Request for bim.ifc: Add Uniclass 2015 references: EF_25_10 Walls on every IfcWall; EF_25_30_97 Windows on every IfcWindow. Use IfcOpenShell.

First a look at what the model holds.

```python
import ifcopenshell

model = ifcopenshell.open("bim.ifc")
print(model.schema)
print("classifications:", [c.Name for c in model.by_type("IfcClassification")])
for ifc_class in ("IfcDoor", "IfcRoof", "IfcStair", "IfcWall", "IfcWindow"):
    print(ifc_class, len(model.by_type(ifc_class)))
```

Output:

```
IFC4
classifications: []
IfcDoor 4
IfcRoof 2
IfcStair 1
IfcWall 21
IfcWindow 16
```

```python
import ifcopenshell
import ifcopenshell.api.classification

model = ifcopenshell.open("bim.ifc")

system = ifcopenshell.api.classification.add_classification(model, classification="Uniclass 2015")

codes = {
    "IfcWall": ("EF_25_10", "Walls"),
    "IfcWindow": ("EF_25_30_97", "Windows"),
}
for ifc_class, (code, name) in codes.items():
    products = model.by_type(ifc_class)
    ifcopenshell.api.classification.add_reference(
        model, products=products, classification=system, identification=code, name=name
    )
    print(code, len(products))

model.write("bim-out.ifc")
```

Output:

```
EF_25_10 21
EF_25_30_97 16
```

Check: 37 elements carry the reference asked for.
